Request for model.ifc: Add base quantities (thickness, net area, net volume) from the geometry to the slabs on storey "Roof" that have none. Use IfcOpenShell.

First a look at what the model holds.

```python
import ifcopenshell
import ifcopenshell.util.element
import ifcopenshell.util.unit

model = ifcopenshell.open("model.ifc")
print(model.schema)
for unit_type in ("LENGTHUNIT", "AREAUNIT", "VOLUMEUNIT"):
    print(unit_type, ifcopenshell.util.unit.calculate_unit_scale(model, unit_type))
storey = next(s for s in model.by_type("IfcBuildingStorey") if s.Name == "Roof")
slabs = [e for e in ifcopenshell.util.element.get_decomposition(storey) if e.is_a("IfcSlab")]
for e in sorted(slabs, key=lambda e: e.id()):
    print(e.id(), e.is_a(), e.Name, list(ifcopenshell.util.element.get_psets(e, qtos_only=True)), sep=" | ")
```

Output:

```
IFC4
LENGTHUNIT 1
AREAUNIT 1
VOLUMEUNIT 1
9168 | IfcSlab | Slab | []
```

```python
import ifcopenshell
import ifcopenshell.api.pset
import ifcopenshell.geom
import ifcopenshell.util.element
import ifcopenshell.util.shape
import ifcopenshell.util.unit

model = ifcopenshell.open("model.ifc")
unit_scale = ifcopenshell.util.unit.calculate_unit_scale(model)
area_scale = ifcopenshell.util.unit.calculate_unit_scale(model, "AREAUNIT")
volume_scale = ifcopenshell.util.unit.calculate_unit_scale(model, "VOLUMEUNIT")
settings = ifcopenshell.geom.settings()

storey = next(s for s in model.by_type("IfcBuildingStorey") if s.Name == "Roof")
slabs = [e for e in ifcopenshell.util.element.get_decomposition(storey) if e.is_a("IfcSlab")]

for e in sorted(slabs, key=lambda e: e.id()):
    if ifcopenshell.util.element.get_psets(e, qtos_only=True, should_inherit=False):
        continue
    # Geometry comes back in metres, in the element's own axes.
    shape = ifcopenshell.geom.create_shape(settings, e)
    values = {
        "Width": ifcopenshell.util.shape.get_z(shape.geometry) / unit_scale,
        "NetArea": ifcopenshell.util.shape.get_footprint_area(shape.geometry) / area_scale,
        "NetVolume": ifcopenshell.util.shape.get_volume(shape.geometry) / volume_scale,
    }
    qto = ifcopenshell.api.pset.add_qto(model, product=e, name="Qto_SlabBaseQuantities")
    ifcopenshell.api.pset.edit_qto(model, qto=qto, properties=values)
    print(e.id(), {k: round(v, 3) for k, v in values.items()})

model.write("model_updated.ifc")
```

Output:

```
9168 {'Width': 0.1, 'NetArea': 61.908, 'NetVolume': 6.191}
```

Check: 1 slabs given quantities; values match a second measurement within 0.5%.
